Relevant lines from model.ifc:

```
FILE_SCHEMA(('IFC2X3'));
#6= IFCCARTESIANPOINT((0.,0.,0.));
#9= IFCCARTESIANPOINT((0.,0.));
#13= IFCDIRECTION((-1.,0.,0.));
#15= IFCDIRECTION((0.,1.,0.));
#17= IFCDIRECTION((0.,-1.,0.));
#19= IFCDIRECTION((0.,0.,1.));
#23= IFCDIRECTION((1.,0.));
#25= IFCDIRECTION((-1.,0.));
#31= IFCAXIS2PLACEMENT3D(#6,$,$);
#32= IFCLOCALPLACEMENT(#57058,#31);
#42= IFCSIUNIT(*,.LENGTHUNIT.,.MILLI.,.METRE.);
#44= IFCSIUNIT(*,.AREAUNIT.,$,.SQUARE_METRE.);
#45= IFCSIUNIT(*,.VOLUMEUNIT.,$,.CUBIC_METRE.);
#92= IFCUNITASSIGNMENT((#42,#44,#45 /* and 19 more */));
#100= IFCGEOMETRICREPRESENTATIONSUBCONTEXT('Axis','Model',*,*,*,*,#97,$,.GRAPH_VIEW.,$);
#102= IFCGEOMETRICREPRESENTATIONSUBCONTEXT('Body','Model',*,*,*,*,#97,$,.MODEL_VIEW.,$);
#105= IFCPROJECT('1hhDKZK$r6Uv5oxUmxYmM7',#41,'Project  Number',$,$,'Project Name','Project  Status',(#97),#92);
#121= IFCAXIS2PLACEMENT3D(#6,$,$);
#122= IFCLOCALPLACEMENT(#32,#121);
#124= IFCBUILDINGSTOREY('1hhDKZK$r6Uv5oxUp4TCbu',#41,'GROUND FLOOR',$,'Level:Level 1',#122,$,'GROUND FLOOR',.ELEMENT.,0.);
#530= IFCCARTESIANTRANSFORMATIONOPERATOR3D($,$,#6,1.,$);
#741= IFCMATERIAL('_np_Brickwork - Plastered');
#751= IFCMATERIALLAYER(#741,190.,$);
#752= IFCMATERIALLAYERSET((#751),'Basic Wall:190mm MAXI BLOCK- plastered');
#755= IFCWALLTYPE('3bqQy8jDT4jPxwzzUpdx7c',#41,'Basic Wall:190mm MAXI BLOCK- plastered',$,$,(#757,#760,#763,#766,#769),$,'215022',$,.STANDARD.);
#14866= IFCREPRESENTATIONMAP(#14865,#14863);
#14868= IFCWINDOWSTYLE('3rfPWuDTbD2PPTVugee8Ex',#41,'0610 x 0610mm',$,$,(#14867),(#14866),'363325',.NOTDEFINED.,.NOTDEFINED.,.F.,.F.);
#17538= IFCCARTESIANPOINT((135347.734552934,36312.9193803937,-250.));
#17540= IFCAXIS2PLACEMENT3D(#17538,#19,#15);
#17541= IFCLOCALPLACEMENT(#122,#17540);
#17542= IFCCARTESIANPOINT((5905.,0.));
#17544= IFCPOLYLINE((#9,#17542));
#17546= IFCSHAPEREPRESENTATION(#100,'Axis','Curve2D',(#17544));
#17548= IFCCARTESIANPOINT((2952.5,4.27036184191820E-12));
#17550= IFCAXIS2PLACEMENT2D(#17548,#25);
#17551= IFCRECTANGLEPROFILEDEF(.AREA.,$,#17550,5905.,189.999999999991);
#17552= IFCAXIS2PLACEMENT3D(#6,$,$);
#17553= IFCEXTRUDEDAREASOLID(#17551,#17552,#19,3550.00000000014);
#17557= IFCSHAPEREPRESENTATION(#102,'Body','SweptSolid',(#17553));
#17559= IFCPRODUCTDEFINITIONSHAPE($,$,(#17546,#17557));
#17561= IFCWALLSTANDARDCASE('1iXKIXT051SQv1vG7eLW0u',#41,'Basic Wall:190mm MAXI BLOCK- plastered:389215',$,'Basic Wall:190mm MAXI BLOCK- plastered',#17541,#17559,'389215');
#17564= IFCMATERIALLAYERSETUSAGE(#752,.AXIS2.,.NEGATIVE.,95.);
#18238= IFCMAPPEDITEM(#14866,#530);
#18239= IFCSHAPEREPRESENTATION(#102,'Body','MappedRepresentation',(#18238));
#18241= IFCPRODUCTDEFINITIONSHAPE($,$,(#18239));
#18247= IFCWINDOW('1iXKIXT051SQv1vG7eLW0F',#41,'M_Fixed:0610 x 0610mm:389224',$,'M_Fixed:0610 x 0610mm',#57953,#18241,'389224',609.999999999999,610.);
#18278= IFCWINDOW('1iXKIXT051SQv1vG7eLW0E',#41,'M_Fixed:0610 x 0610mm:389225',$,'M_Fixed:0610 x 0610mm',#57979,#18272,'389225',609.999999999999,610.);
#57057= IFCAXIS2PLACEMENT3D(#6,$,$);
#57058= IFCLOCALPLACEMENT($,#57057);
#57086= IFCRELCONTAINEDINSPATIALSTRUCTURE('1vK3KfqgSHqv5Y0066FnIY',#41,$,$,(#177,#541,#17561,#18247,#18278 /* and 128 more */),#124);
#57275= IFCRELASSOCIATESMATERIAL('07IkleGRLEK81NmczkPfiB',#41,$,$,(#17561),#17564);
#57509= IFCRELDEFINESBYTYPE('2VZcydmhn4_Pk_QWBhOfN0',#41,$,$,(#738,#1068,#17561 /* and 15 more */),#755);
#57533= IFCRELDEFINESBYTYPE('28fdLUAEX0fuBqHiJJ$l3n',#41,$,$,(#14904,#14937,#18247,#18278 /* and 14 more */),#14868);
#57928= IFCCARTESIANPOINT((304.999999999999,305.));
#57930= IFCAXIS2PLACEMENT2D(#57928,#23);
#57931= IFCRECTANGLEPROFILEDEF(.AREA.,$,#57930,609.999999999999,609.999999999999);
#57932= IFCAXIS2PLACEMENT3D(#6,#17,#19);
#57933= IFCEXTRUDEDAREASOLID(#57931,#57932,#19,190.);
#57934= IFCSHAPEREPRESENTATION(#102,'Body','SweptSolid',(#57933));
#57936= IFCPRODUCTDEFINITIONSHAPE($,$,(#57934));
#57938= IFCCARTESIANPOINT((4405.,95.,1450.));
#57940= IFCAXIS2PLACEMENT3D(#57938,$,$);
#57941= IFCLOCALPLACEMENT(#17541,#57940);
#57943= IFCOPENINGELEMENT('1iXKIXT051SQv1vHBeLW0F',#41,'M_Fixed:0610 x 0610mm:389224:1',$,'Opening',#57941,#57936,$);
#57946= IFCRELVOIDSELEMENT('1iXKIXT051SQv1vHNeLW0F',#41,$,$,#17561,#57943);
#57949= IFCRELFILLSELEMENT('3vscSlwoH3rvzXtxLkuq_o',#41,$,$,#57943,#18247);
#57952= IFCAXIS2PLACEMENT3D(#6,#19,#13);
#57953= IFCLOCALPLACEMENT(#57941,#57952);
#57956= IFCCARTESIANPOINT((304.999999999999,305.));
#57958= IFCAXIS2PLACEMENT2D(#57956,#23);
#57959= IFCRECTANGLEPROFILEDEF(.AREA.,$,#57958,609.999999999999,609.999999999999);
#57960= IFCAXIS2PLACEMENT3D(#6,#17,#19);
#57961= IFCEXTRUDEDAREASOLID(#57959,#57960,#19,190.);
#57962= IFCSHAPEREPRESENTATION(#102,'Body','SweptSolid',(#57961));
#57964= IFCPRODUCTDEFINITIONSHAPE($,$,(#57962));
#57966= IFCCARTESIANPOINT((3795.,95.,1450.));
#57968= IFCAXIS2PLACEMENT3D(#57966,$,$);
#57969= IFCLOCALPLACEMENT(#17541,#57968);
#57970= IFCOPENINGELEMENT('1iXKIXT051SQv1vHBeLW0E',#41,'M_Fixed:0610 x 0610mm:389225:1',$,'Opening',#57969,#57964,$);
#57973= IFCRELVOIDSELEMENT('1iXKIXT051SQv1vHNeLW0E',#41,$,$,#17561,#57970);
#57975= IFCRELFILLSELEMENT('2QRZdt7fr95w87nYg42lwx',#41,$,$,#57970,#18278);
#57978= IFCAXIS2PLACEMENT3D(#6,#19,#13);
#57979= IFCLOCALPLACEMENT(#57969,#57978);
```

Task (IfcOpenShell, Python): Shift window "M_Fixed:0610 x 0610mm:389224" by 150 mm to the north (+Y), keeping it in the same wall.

```python
import ifcopenshell
import ifcopenshell.api.geometry
import ifcopenshell.util.placement

model = ifcopenshell.open("model.ifc")

window = model.by_guid("1iXKIXT051SQv1vG7eLW0F")
opening = window.FillsVoids[0].RelatingOpeningElement
wall = opening.VoidsElements[0].RelatingBuildingElement

wall_matrix = ifcopenshell.util.placement.get_local_placement(wall.ObjectPlacement)
shift = wall_matrix[:3, 0] * 150.0
before = ifcopenshell.util.placement.get_local_placement(window.ObjectPlacement)[:3, 3].copy()

# The window is placed relative to its opening, so it follows when the opening moves.
matrix = ifcopenshell.util.placement.get_local_placement(opening.ObjectPlacement)
matrix[:3, 3] += shift
ifcopenshell.api.geometry.edit_object_placement(
    model, product=opening, matrix=matrix, is_si=False, should_transform_children=True
)

after = ifcopenshell.util.placement.get_local_placement(window.ObjectPlacement)[:3, 3]
print("window moved by", (after - before).round(3) + 0.0)

model.write("model_updated.ifc")
```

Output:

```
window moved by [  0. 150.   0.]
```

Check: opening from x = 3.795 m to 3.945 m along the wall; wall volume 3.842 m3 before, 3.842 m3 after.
